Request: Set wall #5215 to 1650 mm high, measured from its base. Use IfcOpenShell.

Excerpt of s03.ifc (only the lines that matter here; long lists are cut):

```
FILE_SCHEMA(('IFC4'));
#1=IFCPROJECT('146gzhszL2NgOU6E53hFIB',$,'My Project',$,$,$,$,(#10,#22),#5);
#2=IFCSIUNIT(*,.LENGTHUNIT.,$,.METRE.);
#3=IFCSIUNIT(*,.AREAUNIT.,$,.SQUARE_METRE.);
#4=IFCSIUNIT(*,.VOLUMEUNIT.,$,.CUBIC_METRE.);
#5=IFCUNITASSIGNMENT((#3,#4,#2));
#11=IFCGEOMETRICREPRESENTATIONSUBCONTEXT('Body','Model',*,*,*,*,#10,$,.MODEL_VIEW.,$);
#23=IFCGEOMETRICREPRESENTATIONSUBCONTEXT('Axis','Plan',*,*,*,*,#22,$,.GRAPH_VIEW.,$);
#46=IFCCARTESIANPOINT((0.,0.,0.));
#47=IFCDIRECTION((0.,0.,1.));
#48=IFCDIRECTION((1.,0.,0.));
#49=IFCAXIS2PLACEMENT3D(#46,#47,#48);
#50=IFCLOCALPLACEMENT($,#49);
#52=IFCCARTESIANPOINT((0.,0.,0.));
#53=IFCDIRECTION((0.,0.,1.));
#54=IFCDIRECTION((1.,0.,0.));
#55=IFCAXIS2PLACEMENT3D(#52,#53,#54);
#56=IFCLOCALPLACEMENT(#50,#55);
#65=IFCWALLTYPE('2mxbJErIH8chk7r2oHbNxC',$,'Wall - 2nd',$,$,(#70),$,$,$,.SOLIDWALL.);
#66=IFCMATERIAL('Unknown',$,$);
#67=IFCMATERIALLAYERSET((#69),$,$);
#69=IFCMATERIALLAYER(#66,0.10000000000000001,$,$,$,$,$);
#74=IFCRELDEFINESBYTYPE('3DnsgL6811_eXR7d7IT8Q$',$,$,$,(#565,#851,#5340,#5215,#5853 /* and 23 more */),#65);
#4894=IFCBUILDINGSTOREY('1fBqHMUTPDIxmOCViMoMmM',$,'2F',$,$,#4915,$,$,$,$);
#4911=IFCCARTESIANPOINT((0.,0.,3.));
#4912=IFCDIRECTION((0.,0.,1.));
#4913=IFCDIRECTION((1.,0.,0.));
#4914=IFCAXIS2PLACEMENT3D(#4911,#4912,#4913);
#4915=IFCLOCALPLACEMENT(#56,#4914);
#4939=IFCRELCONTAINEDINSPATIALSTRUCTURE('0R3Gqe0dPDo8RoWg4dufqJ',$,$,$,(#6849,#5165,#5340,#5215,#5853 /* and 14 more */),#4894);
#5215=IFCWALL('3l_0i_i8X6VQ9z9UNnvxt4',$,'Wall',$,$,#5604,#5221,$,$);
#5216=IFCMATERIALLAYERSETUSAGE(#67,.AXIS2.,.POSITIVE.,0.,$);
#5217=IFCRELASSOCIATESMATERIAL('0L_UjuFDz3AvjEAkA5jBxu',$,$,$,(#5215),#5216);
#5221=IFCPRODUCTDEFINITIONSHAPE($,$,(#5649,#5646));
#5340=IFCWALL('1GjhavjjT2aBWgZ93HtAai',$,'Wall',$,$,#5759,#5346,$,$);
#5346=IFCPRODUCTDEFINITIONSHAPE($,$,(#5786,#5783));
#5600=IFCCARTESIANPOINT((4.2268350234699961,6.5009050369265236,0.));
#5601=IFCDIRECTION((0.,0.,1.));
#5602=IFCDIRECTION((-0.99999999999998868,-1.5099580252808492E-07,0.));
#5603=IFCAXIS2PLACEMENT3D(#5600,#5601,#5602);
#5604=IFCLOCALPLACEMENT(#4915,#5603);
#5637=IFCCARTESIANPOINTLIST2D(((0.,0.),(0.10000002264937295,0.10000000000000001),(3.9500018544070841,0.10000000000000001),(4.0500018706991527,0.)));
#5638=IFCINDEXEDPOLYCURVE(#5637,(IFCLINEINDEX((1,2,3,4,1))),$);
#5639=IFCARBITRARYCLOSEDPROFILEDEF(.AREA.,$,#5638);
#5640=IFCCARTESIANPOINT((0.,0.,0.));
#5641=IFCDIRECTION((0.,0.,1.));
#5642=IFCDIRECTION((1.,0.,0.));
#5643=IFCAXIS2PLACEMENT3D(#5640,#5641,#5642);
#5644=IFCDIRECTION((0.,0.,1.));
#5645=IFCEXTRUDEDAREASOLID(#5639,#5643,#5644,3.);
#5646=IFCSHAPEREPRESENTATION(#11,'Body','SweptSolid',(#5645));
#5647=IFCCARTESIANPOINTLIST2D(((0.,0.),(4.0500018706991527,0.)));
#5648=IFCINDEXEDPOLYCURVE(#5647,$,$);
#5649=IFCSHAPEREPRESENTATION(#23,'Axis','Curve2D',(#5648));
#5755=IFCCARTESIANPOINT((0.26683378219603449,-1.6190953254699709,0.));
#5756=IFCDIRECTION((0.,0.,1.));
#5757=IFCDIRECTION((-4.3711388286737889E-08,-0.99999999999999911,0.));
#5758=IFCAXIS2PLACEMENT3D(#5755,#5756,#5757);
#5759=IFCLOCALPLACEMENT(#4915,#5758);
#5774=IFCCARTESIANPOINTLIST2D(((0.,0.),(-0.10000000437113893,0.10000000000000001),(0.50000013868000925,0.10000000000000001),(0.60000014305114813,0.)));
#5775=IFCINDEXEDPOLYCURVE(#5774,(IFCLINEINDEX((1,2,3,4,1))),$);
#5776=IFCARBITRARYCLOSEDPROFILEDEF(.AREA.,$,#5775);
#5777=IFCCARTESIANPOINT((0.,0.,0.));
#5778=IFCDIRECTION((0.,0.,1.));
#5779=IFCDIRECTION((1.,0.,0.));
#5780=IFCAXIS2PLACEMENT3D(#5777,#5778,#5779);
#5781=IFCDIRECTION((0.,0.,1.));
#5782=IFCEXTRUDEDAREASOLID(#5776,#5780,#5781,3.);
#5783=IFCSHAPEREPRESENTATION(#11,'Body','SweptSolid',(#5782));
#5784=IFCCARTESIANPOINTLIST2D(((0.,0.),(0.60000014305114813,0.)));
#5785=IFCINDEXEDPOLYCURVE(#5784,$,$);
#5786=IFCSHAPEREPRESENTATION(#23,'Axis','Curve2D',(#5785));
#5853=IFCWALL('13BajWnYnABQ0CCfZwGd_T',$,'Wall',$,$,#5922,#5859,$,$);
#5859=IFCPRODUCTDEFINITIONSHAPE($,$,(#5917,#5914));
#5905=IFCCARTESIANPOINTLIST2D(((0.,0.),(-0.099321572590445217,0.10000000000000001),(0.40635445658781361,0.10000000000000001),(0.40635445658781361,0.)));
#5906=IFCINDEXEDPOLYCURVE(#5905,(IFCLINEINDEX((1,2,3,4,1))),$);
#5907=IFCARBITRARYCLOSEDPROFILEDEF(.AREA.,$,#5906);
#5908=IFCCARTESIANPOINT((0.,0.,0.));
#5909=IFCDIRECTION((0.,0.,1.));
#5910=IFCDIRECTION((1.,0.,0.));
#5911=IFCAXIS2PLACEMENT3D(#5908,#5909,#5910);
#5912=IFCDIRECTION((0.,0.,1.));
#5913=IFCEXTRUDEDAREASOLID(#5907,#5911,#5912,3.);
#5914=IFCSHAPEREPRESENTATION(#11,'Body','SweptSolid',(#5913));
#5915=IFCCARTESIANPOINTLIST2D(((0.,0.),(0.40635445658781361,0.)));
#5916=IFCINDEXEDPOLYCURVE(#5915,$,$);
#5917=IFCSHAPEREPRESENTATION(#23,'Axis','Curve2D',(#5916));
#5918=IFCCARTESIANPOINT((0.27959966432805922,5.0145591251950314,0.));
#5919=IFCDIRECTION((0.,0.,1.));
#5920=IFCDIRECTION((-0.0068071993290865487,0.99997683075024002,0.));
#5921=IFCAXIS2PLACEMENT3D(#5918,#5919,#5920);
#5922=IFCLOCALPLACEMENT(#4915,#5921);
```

```python
import ifcopenshell
import ifcopenshell.geom
import ifcopenshell.util.representation
import ifcopenshell.util.shape
import ifcopenshell.util.unit

model = ifcopenshell.open("s03.ifc")
unit_scale = ifcopenshell.util.unit.calculate_unit_scale(model)
settings = ifcopenshell.geom.settings()


def volume(element):
    """Net volume in cubic metres, openings subtracted."""
    shape = ifcopenshell.geom.create_shape(settings, element)
    return ifcopenshell.util.shape.get_volume(shape.geometry)


wall = model.by_guid("3l_0i_i8X6VQ9z9UNnvxt4")
before = volume(wall)

body = ifcopenshell.util.representation.get_representation(wall, "Model", "Body")
solid = body.Items[0]
old_height = solid.Depth
solid.Depth = 1.65 / unit_scale
after = volume(wall)

print(f"height {old_height:g} -> {solid.Depth:g}, volume {before:.3f} -> {after:.3f} m3")

model.write("s03_edited.ifc")
```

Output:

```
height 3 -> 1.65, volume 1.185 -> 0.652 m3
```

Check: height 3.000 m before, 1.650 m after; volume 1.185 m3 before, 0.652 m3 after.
